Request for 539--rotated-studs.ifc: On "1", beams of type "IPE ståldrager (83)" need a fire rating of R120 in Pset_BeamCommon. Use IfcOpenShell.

First a look at what the model holds.

```python
import ifcopenshell
import ifcopenshell.util.element

model = ifcopenshell.open("539--rotated-studs.ifc")
print(model.schema)
storey = next(s for s in model.by_type("IfcBuildingStorey") if s.Name == "1")
beams = [e for e in ifcopenshell.util.element.get_decomposition(storey) if e.is_a("IfcBeam")]
seen = {}
for e in beams:
    element_type = ifcopenshell.util.element.get_type(e)
    key = (element_type.Name if element_type != e and element_type else None, ifcopenshell.util.element.get_pset(e, "Pset_BeamCommon", "FireRating"))
    seen[key] = seen.get(key, 0) + 1
for (name, value), count in sorted(seen.items(), key=str):
    print(count, "x", name, "|", value)
```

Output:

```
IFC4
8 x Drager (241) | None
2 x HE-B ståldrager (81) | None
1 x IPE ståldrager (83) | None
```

```python
import ifcopenshell
import ifcopenshell.api.pset
import ifcopenshell.util.element

model = ifcopenshell.open("539--rotated-studs.ifc")

storey = next(s for s in model.by_type("IfcBuildingStorey") if s.Name == "1")
beams = [e for e in ifcopenshell.util.element.get_decomposition(storey) if e.is_a("IfcBeam")]

count = 0
for e in beams:
    element_type = ifcopenshell.util.element.get_type(e)
    if element_type in (None, e) or element_type.Name != "IPE ståldrager (83)":
        continue
    # add_pset returns the element's existing set when there is one.
    pset = ifcopenshell.api.pset.add_pset(model, product=e, name="Pset_BeamCommon")
    ifcopenshell.api.pset.edit_pset(model, pset=pset, properties={"FireRating": "R120"})
    count += 1

print(count, "beams updated")

model.write("539--rotated-studs-out.ifc")
```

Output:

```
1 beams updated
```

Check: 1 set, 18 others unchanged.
